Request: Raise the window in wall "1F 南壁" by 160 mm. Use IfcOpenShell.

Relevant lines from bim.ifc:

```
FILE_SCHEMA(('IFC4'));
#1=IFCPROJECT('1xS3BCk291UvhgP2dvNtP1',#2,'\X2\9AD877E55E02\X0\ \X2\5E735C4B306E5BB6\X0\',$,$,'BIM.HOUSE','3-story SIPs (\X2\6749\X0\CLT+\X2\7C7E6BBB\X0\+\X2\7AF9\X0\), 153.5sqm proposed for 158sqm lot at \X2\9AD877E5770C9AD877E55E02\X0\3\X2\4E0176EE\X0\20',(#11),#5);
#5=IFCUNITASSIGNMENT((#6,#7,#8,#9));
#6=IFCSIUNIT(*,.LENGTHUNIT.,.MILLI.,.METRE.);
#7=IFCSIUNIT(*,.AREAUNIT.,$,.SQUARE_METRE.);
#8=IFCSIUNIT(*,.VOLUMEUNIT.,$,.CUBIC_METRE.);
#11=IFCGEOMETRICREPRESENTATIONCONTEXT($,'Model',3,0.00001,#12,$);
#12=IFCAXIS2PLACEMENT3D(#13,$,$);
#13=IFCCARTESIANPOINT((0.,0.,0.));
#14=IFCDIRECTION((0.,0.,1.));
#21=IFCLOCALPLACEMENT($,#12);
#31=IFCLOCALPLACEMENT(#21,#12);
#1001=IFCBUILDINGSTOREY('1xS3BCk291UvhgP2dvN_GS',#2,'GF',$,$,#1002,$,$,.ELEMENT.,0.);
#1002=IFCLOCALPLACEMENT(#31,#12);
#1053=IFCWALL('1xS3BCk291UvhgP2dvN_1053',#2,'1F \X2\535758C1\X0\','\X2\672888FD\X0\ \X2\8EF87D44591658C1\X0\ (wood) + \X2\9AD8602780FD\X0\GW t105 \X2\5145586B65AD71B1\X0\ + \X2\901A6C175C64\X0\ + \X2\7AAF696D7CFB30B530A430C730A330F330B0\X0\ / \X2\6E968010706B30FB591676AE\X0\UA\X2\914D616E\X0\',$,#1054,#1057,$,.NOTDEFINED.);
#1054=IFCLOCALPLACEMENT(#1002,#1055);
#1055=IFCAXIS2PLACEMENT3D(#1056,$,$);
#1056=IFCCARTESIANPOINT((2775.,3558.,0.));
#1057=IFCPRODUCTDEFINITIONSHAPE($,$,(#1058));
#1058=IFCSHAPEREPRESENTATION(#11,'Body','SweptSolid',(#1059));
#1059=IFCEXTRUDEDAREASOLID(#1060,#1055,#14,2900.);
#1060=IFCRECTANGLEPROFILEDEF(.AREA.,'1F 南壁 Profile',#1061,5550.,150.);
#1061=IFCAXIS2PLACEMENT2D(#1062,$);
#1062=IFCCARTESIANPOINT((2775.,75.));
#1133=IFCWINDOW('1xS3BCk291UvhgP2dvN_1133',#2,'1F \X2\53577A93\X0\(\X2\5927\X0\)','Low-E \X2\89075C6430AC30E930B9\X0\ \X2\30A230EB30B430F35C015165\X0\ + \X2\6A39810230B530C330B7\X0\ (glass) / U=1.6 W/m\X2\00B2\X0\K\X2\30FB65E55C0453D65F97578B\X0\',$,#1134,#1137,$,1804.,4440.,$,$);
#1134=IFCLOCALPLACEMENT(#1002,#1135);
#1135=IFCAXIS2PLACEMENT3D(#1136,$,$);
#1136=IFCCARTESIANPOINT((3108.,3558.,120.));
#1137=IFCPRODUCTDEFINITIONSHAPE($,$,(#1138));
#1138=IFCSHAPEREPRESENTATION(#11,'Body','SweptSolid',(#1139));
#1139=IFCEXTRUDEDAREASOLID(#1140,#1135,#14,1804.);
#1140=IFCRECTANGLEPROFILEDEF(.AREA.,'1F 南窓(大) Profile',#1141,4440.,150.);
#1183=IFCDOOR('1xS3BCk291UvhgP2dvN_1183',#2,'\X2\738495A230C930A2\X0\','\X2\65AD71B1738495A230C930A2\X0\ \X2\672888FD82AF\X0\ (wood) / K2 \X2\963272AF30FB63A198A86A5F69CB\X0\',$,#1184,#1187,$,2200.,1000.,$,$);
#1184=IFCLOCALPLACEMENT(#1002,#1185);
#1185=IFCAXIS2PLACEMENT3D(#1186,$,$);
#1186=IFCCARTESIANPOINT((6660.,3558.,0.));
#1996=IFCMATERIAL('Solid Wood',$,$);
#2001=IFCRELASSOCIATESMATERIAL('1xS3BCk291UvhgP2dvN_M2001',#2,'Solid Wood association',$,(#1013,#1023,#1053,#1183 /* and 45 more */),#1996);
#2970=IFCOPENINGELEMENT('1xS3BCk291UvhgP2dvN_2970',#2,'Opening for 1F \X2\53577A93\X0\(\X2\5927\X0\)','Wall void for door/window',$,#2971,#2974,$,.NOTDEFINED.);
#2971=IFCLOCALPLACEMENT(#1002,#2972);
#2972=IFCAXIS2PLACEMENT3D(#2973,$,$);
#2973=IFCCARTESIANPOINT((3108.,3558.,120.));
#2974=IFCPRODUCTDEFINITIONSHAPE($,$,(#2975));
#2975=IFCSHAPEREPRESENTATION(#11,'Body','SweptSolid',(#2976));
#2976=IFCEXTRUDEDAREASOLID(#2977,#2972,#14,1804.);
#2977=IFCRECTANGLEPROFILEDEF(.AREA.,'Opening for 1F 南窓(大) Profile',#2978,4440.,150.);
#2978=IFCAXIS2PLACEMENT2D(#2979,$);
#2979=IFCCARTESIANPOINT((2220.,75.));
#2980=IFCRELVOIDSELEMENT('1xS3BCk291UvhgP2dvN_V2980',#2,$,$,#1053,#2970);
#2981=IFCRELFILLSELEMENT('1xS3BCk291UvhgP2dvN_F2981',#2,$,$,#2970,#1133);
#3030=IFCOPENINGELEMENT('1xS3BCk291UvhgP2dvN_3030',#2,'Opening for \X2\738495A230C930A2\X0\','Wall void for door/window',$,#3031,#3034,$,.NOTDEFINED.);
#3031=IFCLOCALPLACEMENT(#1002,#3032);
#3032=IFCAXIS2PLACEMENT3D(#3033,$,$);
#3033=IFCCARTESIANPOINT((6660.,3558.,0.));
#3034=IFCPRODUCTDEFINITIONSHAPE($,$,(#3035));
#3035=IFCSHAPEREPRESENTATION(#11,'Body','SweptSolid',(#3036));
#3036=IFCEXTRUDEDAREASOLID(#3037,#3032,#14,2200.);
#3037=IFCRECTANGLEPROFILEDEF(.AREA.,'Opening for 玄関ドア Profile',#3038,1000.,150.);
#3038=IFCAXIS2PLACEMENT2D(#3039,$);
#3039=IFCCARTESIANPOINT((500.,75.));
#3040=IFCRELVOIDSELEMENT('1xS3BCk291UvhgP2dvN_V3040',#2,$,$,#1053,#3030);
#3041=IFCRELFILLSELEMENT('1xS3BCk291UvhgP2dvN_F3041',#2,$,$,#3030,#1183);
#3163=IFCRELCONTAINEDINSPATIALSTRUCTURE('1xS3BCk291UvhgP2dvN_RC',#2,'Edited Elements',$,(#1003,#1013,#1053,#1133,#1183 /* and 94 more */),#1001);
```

```python
import numpy as np
import ifcopenshell
import ifcopenshell.api.geometry
import ifcopenshell.util.placement
import ifcopenshell.util.unit

model = ifcopenshell.open("bim.ifc")
unit_scale = ifcopenshell.util.unit.calculate_unit_scale(model)

window = model.by_guid("1xS3BCk291UvhgP2dvN_1133")
opening = window.FillsVoids[0].RelatingOpeningElement
dz = 0.16 / unit_scale

shift = np.array([0.0, 0.0, dz])
# The window is not placed relative to its opening, so move both.
for product in (opening, window):
    matrix = ifcopenshell.util.placement.get_local_placement(product.ObjectPlacement)
    matrix[:3, 3] += shift
    ifcopenshell.api.geometry.edit_object_placement(model, product=product, matrix=matrix, is_si=False)

print(f"moved by {dz * unit_scale:+.3f} m")

model.write("bim_edited.ifc")
```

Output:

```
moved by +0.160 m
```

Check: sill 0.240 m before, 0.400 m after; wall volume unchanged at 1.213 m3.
